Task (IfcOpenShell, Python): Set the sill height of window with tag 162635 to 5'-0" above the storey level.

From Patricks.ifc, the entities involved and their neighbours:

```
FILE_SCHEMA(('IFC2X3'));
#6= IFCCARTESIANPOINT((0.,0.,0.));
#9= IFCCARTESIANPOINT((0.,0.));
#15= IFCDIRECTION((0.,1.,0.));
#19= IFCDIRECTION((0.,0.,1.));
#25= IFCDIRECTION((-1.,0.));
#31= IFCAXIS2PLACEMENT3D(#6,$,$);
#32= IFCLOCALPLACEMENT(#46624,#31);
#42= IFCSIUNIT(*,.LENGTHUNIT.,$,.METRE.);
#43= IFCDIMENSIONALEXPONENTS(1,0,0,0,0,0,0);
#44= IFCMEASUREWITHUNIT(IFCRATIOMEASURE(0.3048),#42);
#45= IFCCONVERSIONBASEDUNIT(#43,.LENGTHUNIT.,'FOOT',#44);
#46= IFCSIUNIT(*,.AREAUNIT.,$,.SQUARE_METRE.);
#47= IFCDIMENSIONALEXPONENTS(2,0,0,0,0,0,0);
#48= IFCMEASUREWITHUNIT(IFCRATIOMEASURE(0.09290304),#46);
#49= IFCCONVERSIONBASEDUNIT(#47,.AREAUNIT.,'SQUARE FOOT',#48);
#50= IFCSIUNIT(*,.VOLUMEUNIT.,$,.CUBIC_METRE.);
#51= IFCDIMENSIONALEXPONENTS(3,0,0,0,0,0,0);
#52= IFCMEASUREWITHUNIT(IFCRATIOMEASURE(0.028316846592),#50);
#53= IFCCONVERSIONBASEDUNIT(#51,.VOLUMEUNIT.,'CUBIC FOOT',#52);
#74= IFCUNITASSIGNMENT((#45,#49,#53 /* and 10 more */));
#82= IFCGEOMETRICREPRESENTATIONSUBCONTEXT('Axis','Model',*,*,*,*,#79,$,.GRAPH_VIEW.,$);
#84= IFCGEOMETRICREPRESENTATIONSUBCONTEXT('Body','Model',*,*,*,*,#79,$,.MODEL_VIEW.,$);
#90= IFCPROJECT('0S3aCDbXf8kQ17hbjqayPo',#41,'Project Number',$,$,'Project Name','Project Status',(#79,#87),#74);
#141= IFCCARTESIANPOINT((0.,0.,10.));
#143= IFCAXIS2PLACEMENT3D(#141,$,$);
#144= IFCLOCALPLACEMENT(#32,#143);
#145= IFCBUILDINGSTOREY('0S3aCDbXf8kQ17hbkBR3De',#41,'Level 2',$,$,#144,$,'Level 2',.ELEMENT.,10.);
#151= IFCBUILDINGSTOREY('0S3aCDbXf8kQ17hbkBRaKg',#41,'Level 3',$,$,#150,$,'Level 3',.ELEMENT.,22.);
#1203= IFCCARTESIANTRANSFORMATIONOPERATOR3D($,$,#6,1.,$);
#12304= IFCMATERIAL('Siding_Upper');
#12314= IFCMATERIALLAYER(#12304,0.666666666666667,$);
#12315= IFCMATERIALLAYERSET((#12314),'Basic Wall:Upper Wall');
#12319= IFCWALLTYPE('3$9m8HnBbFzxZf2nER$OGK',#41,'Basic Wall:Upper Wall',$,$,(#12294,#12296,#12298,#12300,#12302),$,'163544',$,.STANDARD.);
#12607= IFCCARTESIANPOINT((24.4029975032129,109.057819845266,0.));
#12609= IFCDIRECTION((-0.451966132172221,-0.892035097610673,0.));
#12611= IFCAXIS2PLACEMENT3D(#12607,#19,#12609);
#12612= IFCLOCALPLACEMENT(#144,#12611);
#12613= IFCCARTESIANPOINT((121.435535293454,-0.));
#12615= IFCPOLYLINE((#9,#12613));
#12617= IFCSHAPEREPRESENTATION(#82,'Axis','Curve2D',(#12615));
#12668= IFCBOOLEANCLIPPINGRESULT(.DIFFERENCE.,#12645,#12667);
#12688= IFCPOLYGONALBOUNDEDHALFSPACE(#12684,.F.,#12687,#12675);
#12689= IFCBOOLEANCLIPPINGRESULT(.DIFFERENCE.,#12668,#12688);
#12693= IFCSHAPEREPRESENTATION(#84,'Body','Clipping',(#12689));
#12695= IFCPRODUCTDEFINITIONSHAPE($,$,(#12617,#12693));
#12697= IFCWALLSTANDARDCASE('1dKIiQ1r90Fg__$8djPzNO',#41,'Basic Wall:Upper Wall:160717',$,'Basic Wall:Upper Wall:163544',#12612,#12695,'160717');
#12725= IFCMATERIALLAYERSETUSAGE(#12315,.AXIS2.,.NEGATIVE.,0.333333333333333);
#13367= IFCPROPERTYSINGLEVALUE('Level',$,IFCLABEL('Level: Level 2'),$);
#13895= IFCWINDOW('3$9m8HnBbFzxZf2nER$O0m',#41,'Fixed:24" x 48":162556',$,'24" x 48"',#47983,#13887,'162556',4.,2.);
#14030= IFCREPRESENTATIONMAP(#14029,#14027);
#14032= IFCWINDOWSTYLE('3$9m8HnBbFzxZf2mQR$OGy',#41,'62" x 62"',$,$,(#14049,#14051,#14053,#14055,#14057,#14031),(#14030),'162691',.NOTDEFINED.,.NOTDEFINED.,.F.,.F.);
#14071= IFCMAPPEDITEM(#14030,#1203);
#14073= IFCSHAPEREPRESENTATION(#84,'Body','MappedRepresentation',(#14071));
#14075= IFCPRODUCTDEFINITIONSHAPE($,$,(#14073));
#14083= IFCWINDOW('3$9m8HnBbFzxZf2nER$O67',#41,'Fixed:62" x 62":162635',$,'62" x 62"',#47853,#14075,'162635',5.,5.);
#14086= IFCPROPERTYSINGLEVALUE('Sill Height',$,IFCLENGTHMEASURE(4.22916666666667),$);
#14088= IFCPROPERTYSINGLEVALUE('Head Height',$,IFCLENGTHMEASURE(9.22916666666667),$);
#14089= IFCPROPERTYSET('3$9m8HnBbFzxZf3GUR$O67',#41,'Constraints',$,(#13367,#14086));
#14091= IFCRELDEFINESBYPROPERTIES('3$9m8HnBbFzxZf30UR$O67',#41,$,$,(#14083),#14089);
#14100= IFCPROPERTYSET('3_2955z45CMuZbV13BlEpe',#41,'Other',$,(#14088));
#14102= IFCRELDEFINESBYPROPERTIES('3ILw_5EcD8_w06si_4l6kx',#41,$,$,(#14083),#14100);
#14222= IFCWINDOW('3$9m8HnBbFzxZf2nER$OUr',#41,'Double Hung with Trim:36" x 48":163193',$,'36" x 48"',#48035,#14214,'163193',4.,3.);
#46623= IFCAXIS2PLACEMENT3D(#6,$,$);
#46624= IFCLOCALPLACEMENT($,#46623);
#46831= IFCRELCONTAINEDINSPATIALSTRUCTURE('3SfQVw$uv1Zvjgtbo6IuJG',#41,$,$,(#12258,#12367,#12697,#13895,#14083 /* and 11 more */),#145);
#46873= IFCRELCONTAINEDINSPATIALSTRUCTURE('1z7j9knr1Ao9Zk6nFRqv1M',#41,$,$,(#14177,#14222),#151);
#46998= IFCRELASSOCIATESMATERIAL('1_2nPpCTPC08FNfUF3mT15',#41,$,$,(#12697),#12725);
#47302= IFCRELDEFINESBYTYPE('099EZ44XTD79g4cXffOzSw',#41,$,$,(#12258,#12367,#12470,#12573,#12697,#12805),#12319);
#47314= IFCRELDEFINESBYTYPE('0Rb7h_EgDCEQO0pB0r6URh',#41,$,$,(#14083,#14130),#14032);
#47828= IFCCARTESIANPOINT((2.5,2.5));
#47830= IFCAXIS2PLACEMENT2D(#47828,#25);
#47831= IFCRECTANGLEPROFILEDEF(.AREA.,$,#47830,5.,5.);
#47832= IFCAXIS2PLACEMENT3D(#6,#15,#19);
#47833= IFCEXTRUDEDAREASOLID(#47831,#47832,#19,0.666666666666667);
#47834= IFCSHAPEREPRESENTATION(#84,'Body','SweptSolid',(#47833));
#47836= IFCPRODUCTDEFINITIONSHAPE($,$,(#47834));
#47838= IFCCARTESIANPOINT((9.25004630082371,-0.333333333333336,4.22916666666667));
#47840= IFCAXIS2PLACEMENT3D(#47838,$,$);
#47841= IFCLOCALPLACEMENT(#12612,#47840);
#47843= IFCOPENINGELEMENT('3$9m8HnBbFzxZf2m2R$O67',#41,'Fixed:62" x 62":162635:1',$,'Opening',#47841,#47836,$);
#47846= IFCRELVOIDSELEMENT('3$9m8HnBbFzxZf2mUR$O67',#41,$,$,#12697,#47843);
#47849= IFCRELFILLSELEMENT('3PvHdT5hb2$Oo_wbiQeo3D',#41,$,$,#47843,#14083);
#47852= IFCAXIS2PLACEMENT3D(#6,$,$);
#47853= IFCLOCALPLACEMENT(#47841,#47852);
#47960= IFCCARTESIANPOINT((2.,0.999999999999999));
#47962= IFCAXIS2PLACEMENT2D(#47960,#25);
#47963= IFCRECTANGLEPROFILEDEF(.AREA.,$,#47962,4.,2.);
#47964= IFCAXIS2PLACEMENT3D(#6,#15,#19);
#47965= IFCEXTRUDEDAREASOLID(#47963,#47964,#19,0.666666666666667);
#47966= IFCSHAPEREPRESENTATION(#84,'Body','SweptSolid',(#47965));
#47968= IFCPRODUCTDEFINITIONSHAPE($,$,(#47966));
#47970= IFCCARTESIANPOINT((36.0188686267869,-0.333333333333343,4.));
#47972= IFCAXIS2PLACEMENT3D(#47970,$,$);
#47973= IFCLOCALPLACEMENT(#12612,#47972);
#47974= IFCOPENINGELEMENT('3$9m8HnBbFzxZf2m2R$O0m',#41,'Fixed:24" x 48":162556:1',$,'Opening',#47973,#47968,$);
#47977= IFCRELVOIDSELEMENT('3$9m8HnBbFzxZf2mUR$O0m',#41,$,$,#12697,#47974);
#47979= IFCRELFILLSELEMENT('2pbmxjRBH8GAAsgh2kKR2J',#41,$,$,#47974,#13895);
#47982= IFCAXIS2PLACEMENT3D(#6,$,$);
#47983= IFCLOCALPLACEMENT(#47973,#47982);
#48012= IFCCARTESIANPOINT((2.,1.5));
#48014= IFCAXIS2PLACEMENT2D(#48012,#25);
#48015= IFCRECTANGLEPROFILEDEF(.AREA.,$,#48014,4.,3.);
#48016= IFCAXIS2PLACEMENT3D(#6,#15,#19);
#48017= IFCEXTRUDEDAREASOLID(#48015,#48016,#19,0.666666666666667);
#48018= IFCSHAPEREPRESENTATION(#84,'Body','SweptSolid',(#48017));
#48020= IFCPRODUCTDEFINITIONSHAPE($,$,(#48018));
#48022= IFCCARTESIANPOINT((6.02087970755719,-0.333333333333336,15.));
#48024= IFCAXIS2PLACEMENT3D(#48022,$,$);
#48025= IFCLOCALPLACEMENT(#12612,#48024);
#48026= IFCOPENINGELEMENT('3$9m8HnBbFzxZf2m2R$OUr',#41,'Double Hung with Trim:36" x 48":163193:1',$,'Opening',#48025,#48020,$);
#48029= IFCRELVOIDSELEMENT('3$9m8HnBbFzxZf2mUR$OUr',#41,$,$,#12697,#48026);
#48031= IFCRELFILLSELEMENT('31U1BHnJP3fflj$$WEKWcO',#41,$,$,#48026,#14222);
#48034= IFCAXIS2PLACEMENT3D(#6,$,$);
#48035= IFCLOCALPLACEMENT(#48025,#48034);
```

```python
import numpy as np
import ifcopenshell
import ifcopenshell.api.geometry
import ifcopenshell.api.pset
import ifcopenshell.geom
import ifcopenshell.util.element
import ifcopenshell.util.placement
import ifcopenshell.util.shape
import ifcopenshell.util.unit

model = ifcopenshell.open("Patricks.ifc")
unit_scale = ifcopenshell.util.unit.calculate_unit_scale(model)

window = model.by_guid("3$9m8HnBbFzxZf2nER$O67")
opening = window.FillsVoids[0].RelatingOpeningElement
storey = ifcopenshell.util.element.get_container(window, ifc_class="IfcBuildingStorey")
level = ifcopenshell.util.placement.get_local_placement(storey.ObjectPlacement)[2, 3]

# The opening's origin need not be at the sill, so measure its lowest point.
shape = ifcopenshell.geom.create_shape(ifcopenshell.geom.settings(), opening)
bottom = ifcopenshell.util.shape.get_shape_bottom_elevation(shape, shape.geometry) / unit_scale
dz = level + 60 * 0.0254 / unit_scale - bottom

shift = np.array([0.0, 0.0, dz])
# The window is placed relative to its opening, so it follows when the opening moves.
matrix = ifcopenshell.util.placement.get_local_placement(opening.ObjectPlacement)
matrix[:3, 3] += shift
ifcopenshell.api.geometry.edit_object_placement(
    model, product=opening, matrix=matrix, is_si=False, should_transform_children=True
)

# Keep the stored heights in step.
pset = model.by_id(ifcopenshell.util.element.get_pset(window, "Constraints", should_inherit=False)["id"])
ifcopenshell.api.pset.edit_pset(model, pset=pset, properties={
    "Sill Height": model.create_entity("IfcLengthMeasure", ifcopenshell.util.element.get_pset(window, "Constraints", "Sill Height") + dz),
})
pset = model.by_id(ifcopenshell.util.element.get_pset(window, "Other", should_inherit=False)["id"])
ifcopenshell.api.pset.edit_pset(model, pset=pset, properties={
    "Head Height": model.create_entity("IfcLengthMeasure", ifcopenshell.util.element.get_pset(window, "Other", "Head Height") + dz),
})

print(f"moved by {dz * unit_scale:+.3f} m")

model.write("Patricks_v2.ifc")
```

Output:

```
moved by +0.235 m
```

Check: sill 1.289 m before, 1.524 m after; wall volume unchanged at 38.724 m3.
